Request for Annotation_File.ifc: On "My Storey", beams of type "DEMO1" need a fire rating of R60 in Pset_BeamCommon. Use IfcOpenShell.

First a look at what the model holds.

```python
import ifcopenshell
import ifcopenshell.util.element

model = ifcopenshell.open("Annotation_File.ifc")
print(model.schema)
storey = next(s for s in model.by_type("IfcBuildingStorey") if s.Name == "My Storey")
beams = [e for e in ifcopenshell.util.element.get_decomposition(storey) if e.is_a("IfcBeam")]
seen = {}
for e in beams:
    element_type = ifcopenshell.util.element.get_type(e)
    key = (element_type.Name if element_type != e and element_type else None, ifcopenshell.util.element.get_pset(e, "Pset_BeamCommon", "FireRating"))
    seen[key] = seen.get(key, 0) + 1
for (name, value), count in sorted(seen.items(), key=str):
    print(count, "x", name, "|", value)
```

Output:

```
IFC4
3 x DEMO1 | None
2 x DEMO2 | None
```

```python
import ifcopenshell
import ifcopenshell.api.pset
import ifcopenshell.util.element

model = ifcopenshell.open("Annotation_File.ifc")

storey = next(s for s in model.by_type("IfcBuildingStorey") if s.Name == "My Storey")
beams = [e for e in ifcopenshell.util.element.get_decomposition(storey) if e.is_a("IfcBeam")]

count = 0
for e in beams:
    element_type = ifcopenshell.util.element.get_type(e)
    if element_type in (None, e) or element_type.Name != "DEMO1":
        continue
    # add_pset returns the element's existing set when there is one.
    pset = ifcopenshell.api.pset.add_pset(model, product=e, name="Pset_BeamCommon")
    ifcopenshell.api.pset.edit_pset(model, pset=pset, properties={"FireRating": "R60"})
    count += 1

print(count, "beams updated")

model.write("Annotation_File_v2.ifc")
```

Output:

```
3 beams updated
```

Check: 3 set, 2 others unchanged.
